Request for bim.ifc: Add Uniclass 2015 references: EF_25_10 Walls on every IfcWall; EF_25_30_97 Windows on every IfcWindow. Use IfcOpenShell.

First a look at what the model holds.

```python
import ifcopenshell

model = ifcopenshell.open("bim.ifc")
print(model.schema)
print("classifications:", [c.Name for c in model.by_type("IfcClassification")])
for ifc_class in ("IfcDoor", "IfcRoof", "IfcStair", "IfcWall", "IfcWindow"):
    print(ifc_class, len(model.by_type(ifc_class)))
```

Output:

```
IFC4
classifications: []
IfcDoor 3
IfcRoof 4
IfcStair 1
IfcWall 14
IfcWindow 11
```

```python
import ifcopenshell
import ifcopenshell.api.classification

model = ifcopenshell.open("bim.ifc")

system = ifcopenshell.api.classification.add_classification(model, classification="Uniclass 2015")

codes = {
    "IfcWall": ("EF_25_10", "Walls"),
    "IfcWindow": ("EF_25_30_97", "Windows"),
}
for ifc_class, (code, name) in codes.items():
    products = model.by_type(ifc_class)
    ifcopenshell.api.classification.add_reference(
        model, products=products, classification=system, identification=code, name=name
    )
    print(code, len(products))

model.write("bim_v2.ifc")
```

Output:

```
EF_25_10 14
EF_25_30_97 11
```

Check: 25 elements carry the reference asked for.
